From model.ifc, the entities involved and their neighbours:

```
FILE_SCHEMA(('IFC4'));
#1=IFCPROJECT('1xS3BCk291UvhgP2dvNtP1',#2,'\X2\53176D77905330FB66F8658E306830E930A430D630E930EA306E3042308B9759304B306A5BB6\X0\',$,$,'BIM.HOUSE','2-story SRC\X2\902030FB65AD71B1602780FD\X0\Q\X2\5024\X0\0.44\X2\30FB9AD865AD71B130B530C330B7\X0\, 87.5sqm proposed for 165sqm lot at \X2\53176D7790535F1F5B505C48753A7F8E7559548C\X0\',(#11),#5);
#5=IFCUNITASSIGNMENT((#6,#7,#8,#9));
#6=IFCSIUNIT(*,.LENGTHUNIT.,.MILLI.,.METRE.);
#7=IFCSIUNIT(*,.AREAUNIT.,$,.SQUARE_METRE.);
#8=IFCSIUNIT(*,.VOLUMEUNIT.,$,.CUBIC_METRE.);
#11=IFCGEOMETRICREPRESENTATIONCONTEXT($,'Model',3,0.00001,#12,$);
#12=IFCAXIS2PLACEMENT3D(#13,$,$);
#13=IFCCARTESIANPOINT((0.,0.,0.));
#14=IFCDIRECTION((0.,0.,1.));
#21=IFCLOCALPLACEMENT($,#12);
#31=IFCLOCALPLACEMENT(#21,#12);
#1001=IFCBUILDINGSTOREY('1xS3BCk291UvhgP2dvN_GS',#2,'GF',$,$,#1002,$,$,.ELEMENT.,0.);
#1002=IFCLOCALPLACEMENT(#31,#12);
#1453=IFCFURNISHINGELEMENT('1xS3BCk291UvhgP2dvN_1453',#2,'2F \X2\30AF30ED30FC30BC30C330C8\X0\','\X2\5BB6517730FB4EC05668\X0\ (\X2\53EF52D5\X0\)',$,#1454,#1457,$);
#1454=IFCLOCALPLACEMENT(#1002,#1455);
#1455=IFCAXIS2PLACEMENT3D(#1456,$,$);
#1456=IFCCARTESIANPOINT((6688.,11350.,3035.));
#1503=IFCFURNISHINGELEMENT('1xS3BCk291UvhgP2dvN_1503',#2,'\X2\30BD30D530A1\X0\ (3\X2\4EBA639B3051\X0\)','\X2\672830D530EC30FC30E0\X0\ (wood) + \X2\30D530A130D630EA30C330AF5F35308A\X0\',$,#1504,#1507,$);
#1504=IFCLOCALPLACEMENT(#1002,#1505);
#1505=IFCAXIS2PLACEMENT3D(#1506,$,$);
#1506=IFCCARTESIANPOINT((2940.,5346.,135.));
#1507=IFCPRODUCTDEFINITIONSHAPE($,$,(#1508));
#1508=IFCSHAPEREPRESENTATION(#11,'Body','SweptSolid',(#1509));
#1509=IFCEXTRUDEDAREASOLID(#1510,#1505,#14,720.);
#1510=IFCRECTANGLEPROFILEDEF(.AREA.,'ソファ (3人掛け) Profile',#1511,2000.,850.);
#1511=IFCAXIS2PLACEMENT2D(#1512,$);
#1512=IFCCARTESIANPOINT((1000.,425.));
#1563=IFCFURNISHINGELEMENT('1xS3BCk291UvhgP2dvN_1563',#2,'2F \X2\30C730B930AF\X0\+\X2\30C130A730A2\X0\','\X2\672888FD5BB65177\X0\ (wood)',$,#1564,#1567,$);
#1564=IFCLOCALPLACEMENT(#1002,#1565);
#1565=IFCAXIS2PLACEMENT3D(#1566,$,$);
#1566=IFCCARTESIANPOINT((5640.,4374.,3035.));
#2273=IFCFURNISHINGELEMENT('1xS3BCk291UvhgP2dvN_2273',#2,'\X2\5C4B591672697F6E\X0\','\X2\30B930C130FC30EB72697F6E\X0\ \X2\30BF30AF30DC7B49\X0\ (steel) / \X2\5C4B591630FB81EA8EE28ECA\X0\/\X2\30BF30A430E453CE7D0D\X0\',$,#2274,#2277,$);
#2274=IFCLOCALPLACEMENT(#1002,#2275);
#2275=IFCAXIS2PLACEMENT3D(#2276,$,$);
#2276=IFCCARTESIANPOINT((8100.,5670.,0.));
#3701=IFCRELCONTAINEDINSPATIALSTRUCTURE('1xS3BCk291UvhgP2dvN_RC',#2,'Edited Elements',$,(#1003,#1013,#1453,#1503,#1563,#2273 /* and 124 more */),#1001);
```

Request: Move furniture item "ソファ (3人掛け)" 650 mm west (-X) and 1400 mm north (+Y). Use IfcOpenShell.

```python
import ifcopenshell
import ifcopenshell.api.geometry
import ifcopenshell.util.placement
import ifcopenshell.util.unit

model = ifcopenshell.open("model.ifc")
unit_scale = ifcopenshell.util.unit.calculate_unit_scale(model)

item = model.by_guid("1xS3BCk291UvhgP2dvN_1503")
matrix = ifcopenshell.util.placement.get_local_placement(item.ObjectPlacement)
matrix[0, 3] -= 0.65 / unit_scale
matrix[1, 3] += 1.4 / unit_scale
ifcopenshell.api.geometry.edit_object_placement(model, product=item, matrix=matrix, is_si=False)

print(ifcopenshell.util.placement.get_local_placement(item.ObjectPlacement).round(3) + 0.0)

model.write("model-out.ifc")
```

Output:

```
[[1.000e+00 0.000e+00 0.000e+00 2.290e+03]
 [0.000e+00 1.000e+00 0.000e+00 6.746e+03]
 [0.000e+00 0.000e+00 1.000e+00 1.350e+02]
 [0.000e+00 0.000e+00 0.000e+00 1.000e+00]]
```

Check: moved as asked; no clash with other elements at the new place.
